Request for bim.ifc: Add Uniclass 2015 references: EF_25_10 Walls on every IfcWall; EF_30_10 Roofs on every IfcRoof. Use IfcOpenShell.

First a look at what the model holds.

```python
import ifcopenshell

model = ifcopenshell.open("bim.ifc")
print(model.schema)
print("classifications:", [c.Name for c in model.by_type("IfcClassification")])
for ifc_class in ("IfcDoor", "IfcRoof", "IfcStair", "IfcWall", "IfcWindow"):
    print(ifc_class, len(model.by_type(ifc_class)))
```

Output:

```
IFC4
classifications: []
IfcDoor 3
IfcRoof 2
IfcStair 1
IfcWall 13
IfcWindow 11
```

```python
import ifcopenshell
import ifcopenshell.api.classification

model = ifcopenshell.open("bim.ifc")

system = ifcopenshell.api.classification.add_classification(model, classification="Uniclass 2015")

codes = {
    "IfcWall": ("EF_25_10", "Walls"),
    "IfcRoof": ("EF_30_10", "Roofs"),
}
for ifc_class, (code, name) in codes.items():
    products = model.by_type(ifc_class)
    ifcopenshell.api.classification.add_reference(
        model, products=products, classification=system, identification=code, name=name
    )
    print(code, len(products))

model.write("bim_v2.ifc")
```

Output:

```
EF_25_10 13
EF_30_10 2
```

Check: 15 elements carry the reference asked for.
